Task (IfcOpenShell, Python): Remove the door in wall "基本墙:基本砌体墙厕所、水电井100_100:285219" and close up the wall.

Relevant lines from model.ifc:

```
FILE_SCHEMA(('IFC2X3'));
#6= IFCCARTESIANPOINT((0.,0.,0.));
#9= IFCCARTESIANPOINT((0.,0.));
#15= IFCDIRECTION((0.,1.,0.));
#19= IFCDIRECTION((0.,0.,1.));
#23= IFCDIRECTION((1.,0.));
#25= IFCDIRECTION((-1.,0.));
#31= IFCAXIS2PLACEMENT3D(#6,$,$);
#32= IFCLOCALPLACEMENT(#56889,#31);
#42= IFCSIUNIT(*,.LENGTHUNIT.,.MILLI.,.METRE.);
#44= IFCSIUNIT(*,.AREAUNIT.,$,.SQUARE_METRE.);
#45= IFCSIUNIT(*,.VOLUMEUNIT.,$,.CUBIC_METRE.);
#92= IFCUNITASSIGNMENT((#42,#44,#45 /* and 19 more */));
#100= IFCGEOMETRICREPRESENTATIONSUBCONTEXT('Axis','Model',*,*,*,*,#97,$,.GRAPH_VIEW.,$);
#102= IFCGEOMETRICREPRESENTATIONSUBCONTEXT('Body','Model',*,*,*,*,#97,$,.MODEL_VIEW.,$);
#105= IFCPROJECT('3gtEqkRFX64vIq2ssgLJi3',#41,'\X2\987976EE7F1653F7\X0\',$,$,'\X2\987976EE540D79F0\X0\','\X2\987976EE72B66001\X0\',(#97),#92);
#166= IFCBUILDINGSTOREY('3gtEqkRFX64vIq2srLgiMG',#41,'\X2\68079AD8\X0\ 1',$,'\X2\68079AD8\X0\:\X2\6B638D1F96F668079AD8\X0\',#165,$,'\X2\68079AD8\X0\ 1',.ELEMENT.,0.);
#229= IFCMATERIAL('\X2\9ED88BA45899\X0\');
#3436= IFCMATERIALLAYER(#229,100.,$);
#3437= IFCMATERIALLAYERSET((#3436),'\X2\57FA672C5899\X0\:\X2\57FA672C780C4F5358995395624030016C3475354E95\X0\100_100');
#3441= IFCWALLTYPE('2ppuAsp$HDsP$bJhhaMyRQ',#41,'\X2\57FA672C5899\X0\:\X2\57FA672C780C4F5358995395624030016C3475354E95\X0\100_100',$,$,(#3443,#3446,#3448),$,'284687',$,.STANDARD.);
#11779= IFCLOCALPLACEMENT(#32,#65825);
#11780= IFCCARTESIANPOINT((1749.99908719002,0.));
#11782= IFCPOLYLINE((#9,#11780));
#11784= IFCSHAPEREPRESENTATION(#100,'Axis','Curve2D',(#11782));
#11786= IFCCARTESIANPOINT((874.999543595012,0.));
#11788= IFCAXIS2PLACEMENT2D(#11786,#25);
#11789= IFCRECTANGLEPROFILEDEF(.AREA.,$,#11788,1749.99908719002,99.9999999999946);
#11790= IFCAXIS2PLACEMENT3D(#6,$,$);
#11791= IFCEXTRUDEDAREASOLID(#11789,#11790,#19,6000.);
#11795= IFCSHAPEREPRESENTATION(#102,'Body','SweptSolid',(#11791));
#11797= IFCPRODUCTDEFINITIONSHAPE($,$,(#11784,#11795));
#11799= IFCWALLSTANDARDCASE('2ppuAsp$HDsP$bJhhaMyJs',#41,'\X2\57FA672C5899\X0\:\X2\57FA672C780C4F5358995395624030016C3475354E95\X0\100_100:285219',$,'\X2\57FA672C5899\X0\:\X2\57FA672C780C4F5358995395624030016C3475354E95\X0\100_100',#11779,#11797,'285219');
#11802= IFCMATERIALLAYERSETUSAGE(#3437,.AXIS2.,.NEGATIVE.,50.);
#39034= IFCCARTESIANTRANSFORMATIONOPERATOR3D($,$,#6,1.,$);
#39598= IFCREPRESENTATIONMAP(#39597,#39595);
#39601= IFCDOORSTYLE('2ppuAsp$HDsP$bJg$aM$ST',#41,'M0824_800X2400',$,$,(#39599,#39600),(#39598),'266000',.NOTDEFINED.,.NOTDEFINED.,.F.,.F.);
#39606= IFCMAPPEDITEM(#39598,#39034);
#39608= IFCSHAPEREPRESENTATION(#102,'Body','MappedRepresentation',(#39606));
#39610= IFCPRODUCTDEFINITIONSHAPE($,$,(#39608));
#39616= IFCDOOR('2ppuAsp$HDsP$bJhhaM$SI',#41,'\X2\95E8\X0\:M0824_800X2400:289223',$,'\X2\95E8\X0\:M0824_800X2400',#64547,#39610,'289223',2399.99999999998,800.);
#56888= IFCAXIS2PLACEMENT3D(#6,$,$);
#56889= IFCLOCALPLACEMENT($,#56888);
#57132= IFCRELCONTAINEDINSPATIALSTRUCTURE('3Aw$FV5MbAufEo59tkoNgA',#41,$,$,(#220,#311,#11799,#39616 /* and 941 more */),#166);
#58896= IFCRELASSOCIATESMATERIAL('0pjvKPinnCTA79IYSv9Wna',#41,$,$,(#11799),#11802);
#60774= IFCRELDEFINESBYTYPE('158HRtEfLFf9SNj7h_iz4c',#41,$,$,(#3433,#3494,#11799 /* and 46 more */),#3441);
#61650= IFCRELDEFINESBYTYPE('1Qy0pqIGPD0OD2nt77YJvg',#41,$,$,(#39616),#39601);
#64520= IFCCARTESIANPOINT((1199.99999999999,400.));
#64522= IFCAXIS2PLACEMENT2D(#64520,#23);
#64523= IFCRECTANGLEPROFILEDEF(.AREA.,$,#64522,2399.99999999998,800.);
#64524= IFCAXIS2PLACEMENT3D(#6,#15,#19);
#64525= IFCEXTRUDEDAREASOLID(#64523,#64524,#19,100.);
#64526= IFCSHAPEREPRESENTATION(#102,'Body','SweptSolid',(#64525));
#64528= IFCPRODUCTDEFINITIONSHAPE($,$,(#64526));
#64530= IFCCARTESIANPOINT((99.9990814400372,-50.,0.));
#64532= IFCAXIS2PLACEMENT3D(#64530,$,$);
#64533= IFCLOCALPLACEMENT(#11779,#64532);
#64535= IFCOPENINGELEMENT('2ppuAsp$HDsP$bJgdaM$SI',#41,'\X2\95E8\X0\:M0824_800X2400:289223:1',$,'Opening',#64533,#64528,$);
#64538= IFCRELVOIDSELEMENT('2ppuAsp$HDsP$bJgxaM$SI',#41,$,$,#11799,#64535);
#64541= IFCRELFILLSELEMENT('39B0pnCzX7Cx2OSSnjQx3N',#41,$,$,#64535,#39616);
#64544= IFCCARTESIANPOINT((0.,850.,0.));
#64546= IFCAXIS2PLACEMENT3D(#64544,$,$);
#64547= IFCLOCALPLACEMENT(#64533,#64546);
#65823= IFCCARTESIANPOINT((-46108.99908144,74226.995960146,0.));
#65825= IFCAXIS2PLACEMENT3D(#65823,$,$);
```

```python
import ifcopenshell
import ifcopenshell.api.feature
import ifcopenshell.api.root
import ifcopenshell.geom
import ifcopenshell.util.shape

model = ifcopenshell.open("model.ifc")
settings = ifcopenshell.geom.settings()


def volume(element):
    """Net volume in cubic metres, openings subtracted."""
    shape = ifcopenshell.geom.create_shape(settings, element)
    return ifcopenshell.util.shape.get_volume(shape.geometry)


door = model.by_guid("2ppuAsp$HDsP$bJhhaM$SI")
opening = door.FillsVoids[0].RelatingOpeningElement
wall = opening.VoidsElements[0].RelatingBuildingElement
before = volume(wall)

ifcopenshell.api.root.remove_product(model, product=door)
ifcopenshell.api.feature.remove_feature(model, feature=opening)

after = volume(wall)

print(f"wall volume {before:.3f} -> {after:.3f} m3")

model.write("model_edited.ifc")
```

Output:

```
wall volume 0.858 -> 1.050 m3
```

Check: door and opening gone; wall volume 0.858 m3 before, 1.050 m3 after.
